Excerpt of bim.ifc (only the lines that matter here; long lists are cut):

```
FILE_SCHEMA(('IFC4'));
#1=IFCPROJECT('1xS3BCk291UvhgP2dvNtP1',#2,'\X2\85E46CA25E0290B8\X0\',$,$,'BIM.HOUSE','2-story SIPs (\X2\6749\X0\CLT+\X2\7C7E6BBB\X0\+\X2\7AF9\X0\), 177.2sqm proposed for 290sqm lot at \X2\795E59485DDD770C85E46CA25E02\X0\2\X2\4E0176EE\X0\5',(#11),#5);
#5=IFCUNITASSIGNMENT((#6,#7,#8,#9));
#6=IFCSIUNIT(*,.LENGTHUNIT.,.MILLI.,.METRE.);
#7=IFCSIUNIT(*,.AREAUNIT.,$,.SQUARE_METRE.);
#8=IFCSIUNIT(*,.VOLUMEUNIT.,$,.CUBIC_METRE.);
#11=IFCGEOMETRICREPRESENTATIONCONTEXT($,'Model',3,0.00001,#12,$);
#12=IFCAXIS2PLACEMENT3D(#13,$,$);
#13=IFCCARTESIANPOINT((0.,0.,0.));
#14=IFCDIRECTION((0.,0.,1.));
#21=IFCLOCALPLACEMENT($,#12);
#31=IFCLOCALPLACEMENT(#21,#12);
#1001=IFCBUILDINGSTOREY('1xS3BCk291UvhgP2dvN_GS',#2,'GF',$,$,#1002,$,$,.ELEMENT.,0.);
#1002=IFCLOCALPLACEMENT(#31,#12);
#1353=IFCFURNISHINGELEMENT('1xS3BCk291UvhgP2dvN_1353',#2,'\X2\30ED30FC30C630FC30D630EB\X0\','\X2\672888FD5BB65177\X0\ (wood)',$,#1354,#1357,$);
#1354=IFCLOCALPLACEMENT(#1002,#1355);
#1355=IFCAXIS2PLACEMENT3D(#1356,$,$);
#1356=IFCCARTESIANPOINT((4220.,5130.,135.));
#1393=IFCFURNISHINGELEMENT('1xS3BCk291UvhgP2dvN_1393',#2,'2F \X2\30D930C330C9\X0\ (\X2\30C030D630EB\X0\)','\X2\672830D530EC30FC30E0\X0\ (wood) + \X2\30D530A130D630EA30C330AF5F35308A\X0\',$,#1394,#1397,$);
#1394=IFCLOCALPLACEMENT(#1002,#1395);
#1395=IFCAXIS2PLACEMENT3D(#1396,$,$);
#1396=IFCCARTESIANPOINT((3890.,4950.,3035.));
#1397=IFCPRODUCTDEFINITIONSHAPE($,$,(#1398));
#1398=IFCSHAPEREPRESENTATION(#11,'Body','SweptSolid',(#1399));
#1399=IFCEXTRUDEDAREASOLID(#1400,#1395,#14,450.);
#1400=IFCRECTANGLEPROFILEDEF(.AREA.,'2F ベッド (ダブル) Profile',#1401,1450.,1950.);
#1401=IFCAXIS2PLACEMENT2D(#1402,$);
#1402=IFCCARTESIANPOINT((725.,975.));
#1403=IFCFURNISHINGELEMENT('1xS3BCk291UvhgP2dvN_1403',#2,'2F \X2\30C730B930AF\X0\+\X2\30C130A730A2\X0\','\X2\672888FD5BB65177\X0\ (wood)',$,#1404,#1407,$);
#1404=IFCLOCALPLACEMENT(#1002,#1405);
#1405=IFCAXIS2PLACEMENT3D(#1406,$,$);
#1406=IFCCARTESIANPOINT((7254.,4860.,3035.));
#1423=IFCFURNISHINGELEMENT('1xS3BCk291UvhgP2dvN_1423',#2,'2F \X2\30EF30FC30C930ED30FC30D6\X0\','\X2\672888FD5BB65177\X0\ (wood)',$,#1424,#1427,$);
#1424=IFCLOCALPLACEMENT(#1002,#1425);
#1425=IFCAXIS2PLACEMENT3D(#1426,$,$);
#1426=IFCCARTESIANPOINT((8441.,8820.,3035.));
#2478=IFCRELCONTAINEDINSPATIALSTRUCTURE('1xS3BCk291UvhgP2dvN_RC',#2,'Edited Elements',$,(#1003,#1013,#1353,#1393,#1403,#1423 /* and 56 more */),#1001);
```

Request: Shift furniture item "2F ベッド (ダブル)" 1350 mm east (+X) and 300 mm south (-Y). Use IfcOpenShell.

```python
import ifcopenshell
import ifcopenshell.api.geometry
import ifcopenshell.util.placement

model = ifcopenshell.open("bim.ifc")

item = model.by_guid("1xS3BCk291UvhgP2dvN_1393")
matrix = ifcopenshell.util.placement.get_local_placement(item.ObjectPlacement)
matrix[0, 3] += 1350.0
matrix[1, 3] -= 300.0
ifcopenshell.api.geometry.edit_object_placement(model, product=item, matrix=matrix, is_si=False)

print(ifcopenshell.util.placement.get_local_placement(item.ObjectPlacement).round(3) + 0.0)

model.write("bim_updated.ifc")
```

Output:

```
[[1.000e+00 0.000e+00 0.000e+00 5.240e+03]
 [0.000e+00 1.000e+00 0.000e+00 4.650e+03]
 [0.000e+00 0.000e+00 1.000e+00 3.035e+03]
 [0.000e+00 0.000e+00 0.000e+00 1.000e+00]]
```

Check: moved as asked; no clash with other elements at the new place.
